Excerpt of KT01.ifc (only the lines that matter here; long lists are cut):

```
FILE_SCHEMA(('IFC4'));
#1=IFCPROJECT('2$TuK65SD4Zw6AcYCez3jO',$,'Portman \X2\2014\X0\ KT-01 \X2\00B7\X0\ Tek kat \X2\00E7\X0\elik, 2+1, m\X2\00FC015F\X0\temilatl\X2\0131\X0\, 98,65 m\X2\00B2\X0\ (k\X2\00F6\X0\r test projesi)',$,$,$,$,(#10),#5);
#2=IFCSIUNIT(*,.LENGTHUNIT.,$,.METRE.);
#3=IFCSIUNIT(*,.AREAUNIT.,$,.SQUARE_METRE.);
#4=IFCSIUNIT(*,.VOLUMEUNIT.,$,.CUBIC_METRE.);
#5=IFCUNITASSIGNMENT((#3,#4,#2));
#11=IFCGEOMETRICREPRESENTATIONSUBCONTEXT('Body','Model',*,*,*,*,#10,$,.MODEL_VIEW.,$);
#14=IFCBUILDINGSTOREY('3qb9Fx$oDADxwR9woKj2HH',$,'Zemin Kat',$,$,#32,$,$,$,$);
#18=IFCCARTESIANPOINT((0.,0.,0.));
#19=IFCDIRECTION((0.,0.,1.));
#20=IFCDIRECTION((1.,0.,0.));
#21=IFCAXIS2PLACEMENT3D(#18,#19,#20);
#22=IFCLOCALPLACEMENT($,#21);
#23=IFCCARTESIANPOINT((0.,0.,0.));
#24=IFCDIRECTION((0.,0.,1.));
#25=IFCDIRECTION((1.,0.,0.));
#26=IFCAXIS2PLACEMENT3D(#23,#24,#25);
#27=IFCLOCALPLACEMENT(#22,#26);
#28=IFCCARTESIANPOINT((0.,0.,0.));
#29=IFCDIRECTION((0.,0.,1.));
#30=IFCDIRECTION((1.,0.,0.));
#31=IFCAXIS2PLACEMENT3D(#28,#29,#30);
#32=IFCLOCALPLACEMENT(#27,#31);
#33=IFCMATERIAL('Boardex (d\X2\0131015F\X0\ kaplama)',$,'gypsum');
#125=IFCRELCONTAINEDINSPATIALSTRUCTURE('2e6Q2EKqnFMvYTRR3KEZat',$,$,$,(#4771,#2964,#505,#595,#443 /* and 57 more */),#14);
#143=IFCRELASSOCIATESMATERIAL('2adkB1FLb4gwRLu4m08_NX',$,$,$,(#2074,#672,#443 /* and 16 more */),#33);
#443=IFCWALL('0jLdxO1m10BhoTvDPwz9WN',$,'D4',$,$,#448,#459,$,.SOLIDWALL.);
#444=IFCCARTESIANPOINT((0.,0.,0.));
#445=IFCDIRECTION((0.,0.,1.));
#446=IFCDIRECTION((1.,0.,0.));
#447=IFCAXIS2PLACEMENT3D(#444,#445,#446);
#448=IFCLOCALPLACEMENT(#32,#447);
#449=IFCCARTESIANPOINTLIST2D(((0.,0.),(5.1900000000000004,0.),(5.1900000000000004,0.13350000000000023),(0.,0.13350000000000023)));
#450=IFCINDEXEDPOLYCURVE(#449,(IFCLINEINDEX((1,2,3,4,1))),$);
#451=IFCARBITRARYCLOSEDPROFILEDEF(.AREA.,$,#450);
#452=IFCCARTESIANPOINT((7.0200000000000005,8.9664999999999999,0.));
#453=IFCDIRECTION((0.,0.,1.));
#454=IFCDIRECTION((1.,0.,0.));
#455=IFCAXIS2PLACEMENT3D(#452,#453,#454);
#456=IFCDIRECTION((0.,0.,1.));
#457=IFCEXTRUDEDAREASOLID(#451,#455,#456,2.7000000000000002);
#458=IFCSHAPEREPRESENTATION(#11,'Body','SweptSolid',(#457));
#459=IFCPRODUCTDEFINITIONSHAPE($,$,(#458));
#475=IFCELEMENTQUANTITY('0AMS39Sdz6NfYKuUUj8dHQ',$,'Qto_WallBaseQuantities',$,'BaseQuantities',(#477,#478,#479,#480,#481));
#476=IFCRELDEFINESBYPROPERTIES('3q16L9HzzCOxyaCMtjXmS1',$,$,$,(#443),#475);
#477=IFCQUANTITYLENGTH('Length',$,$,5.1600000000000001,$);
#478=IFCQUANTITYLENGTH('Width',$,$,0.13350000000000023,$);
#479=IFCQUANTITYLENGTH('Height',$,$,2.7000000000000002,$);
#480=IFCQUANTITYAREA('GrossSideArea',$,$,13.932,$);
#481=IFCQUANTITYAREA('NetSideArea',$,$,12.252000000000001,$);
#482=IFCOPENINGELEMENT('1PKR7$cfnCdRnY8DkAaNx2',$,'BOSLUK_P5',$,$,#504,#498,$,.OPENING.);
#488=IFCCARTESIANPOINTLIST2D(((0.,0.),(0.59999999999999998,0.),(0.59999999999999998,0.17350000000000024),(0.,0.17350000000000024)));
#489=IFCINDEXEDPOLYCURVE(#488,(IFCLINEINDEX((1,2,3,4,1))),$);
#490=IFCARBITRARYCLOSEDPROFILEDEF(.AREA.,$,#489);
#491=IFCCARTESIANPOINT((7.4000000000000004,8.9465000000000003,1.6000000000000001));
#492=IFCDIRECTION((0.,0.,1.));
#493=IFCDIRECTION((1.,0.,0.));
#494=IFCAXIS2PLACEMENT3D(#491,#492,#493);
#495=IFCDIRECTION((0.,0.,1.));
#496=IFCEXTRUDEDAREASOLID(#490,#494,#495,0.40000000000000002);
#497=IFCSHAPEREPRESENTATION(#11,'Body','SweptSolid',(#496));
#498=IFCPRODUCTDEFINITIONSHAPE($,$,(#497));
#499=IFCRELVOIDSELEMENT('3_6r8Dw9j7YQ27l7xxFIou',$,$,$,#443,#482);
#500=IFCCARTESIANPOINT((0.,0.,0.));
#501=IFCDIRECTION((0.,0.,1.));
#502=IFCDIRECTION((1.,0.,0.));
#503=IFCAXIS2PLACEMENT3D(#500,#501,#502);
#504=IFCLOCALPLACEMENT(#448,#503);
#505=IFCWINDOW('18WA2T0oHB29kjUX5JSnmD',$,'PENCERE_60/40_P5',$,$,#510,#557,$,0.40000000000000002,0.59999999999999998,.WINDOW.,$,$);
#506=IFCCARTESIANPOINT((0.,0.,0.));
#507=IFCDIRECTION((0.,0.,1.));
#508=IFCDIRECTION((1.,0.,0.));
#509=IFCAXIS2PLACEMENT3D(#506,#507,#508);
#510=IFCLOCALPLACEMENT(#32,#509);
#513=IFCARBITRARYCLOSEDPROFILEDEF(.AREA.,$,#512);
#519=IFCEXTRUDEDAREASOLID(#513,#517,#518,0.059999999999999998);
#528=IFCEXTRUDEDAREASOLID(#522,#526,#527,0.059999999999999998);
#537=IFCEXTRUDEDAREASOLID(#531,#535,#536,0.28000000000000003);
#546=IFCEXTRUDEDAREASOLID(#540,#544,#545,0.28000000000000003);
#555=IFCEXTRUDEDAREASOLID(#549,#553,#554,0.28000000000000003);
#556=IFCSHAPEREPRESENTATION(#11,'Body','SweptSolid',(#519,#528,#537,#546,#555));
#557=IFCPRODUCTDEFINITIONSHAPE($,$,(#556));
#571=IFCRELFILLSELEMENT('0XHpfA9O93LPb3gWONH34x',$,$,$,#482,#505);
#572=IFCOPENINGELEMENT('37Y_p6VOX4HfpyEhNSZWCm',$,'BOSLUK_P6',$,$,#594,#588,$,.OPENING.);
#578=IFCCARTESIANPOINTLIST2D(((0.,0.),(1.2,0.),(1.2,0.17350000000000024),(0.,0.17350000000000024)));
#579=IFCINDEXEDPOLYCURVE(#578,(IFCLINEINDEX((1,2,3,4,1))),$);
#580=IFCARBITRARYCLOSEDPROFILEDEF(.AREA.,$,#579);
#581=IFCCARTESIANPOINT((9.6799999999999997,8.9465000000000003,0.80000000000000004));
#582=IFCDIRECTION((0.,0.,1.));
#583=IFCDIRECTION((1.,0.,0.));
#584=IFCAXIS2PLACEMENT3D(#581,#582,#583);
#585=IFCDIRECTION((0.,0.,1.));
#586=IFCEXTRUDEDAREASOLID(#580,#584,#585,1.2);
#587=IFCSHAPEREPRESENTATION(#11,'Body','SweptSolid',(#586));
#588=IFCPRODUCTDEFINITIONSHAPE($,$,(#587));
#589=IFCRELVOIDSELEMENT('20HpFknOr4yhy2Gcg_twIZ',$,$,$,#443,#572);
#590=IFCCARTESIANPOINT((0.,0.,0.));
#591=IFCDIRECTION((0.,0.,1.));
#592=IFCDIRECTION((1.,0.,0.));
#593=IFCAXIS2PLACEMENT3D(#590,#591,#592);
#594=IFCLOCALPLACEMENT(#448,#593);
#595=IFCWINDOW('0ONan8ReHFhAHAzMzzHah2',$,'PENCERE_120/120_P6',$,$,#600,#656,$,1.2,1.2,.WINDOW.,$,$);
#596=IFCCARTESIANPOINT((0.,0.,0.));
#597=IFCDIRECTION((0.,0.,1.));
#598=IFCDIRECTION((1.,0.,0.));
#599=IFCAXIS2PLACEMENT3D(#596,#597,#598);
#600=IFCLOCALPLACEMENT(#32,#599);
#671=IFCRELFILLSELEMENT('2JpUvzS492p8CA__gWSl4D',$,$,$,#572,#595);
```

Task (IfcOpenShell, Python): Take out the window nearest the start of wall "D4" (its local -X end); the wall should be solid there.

```python
import ifcopenshell
import ifcopenshell.api.feature
import ifcopenshell.api.pset
import ifcopenshell.api.root
import ifcopenshell.geom
import ifcopenshell.util.element
import ifcopenshell.util.shape
import ifcopenshell.util.unit

model = ifcopenshell.open("KT01.ifc")
area_scale = ifcopenshell.util.unit.calculate_unit_scale(model, "AREAUNIT")
settings = ifcopenshell.geom.settings()


def volume(element):
    """Net volume in cubic metres, openings subtracted."""
    shape = ifcopenshell.geom.create_shape(settings, element)
    return ifcopenshell.util.shape.get_volume(shape.geometry)


window = model.by_guid("18WA2T0oHB29kjUX5JSnmD")
opening = window.FillsVoids[0].RelatingOpeningElement
wall = opening.VoidsElements[0].RelatingBuildingElement
before = volume(wall)

ifcopenshell.api.root.remove_product(model, product=window)
ifcopenshell.api.feature.remove_feature(model, feature=opening)

after = volume(wall)
thickness = 0.1335  # wall thickness in metres

# Update the wall's stored quantities.
qto = model.by_id(ifcopenshell.util.element.get_pset(wall, "Qto_WallBaseQuantities", should_inherit=False)["id"])
ifcopenshell.api.pset.edit_qto(model, qto=qto, properties={"NetSideArea": after / thickness / area_scale})

print(f"wall volume {before:.3f} -> {after:.3f} m3")

model.write("KT01-out.ifc")
```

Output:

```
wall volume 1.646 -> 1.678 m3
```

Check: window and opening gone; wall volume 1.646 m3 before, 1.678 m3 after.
